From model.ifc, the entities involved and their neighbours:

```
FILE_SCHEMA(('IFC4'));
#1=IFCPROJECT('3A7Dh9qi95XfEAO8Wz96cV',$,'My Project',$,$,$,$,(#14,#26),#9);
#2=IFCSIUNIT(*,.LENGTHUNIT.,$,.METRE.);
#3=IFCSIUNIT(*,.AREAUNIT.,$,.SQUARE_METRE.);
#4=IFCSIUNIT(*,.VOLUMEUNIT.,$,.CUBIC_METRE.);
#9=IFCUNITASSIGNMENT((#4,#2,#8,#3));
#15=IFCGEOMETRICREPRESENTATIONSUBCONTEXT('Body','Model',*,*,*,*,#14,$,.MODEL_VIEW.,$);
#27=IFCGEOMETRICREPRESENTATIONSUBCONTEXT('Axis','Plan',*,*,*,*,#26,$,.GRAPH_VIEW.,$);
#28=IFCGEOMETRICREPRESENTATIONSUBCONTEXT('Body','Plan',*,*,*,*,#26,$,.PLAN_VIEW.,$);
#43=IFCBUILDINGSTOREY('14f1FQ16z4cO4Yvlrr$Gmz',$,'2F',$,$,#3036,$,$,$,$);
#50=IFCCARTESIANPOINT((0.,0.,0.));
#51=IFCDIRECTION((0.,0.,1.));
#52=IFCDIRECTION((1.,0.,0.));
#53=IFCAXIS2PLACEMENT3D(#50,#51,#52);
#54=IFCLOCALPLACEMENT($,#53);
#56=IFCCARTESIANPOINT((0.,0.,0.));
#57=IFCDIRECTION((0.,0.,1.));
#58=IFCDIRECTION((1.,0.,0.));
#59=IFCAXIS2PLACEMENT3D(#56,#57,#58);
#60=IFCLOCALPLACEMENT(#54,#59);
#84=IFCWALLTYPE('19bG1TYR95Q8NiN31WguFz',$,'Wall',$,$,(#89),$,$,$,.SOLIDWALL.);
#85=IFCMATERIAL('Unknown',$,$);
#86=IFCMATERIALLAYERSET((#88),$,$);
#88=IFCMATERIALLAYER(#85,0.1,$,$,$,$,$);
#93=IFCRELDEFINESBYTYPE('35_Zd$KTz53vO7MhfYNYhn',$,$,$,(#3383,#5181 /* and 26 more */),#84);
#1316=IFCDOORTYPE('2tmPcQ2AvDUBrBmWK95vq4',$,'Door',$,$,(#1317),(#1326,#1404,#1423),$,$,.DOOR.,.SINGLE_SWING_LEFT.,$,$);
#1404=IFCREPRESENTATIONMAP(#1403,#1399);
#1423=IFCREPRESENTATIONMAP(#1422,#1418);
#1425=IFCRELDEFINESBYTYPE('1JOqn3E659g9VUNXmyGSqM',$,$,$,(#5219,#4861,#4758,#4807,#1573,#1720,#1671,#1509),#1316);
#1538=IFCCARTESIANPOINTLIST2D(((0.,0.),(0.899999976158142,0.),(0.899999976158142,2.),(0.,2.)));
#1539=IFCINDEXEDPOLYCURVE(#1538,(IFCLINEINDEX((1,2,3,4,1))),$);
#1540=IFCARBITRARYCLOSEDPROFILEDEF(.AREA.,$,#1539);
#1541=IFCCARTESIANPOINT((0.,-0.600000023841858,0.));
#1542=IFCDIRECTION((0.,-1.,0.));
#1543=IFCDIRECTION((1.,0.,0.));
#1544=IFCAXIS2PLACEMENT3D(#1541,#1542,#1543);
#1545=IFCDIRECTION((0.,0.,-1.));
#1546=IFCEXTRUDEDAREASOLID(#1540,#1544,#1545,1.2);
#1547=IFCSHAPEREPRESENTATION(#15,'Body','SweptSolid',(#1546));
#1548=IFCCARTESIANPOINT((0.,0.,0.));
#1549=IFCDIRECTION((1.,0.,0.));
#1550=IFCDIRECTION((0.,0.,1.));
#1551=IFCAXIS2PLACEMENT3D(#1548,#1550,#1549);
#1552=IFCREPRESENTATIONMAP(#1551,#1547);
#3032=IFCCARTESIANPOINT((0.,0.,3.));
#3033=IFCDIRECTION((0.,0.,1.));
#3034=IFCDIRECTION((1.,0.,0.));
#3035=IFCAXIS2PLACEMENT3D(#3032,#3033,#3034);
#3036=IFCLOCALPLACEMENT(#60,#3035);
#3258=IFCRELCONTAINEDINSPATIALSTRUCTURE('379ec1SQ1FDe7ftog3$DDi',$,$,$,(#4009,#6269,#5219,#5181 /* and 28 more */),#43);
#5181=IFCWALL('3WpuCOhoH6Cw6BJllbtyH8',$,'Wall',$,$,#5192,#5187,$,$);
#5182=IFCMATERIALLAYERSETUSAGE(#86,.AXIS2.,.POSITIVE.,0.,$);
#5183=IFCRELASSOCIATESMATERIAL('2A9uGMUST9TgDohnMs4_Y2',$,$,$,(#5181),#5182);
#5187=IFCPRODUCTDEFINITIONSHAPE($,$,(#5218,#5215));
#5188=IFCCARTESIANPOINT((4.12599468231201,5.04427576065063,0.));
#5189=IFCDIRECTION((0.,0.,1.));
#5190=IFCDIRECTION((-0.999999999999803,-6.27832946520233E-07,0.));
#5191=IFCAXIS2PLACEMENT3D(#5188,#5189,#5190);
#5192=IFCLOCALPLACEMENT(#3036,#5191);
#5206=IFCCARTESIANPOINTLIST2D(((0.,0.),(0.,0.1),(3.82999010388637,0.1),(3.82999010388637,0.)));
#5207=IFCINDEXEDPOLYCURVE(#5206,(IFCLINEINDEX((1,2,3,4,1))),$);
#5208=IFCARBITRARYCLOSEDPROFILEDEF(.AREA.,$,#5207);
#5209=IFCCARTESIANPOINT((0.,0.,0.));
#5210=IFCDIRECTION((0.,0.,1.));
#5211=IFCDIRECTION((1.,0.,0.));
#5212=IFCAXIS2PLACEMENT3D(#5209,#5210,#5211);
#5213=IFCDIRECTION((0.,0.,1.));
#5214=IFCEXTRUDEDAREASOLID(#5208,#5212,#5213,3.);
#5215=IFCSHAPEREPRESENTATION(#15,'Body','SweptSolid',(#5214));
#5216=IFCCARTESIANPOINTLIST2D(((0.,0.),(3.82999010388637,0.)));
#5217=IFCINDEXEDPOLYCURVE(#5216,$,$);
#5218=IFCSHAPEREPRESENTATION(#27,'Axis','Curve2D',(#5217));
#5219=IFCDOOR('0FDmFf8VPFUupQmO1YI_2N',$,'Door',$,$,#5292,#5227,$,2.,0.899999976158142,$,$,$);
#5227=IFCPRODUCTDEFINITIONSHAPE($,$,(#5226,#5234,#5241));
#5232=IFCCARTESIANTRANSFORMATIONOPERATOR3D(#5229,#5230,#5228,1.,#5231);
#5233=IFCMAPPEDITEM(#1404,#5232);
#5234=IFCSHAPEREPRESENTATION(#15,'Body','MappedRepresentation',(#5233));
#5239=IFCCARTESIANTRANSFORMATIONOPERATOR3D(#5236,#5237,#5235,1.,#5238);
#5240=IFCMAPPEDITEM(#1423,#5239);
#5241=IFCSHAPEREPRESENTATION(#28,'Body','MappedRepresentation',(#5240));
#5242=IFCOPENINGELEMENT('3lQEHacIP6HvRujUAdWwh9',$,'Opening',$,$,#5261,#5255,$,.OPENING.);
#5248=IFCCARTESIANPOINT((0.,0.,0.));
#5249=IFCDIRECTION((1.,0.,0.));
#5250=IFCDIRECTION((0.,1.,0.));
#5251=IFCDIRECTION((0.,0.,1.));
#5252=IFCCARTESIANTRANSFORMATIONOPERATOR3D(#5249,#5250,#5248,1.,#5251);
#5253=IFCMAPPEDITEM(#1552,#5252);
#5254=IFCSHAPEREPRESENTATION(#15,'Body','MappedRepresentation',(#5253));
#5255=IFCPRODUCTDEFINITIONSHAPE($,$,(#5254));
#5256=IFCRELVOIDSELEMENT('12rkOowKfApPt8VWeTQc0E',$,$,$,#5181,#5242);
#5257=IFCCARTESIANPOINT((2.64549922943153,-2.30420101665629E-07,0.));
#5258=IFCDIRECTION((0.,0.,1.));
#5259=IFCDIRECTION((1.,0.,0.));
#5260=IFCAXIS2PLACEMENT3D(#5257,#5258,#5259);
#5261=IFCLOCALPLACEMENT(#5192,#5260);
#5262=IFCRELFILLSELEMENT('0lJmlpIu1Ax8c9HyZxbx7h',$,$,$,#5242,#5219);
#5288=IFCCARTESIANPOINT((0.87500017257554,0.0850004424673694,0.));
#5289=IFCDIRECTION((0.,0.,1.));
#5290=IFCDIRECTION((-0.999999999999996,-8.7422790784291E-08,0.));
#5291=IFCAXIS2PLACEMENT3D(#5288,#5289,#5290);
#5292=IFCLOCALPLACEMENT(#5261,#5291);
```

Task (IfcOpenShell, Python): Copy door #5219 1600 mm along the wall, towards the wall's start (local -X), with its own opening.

```python
import ifcopenshell
import ifcopenshell.api.feature
import ifcopenshell.api.geometry
import ifcopenshell.api.root
import ifcopenshell.geom
import ifcopenshell.util.element
import ifcopenshell.util.placement
import ifcopenshell.util.shape

model = ifcopenshell.open("model.ifc")
settings = ifcopenshell.geom.settings()


def volume(element):
    """Net volume in cubic metres, openings subtracted."""
    shape = ifcopenshell.geom.create_shape(settings, element)
    return ifcopenshell.util.shape.get_volume(shape.geometry)


door = model.by_guid("0FDmFf8VPFUupQmO1YI_2N")
opening = door.FillsVoids[0].RelatingOpeningElement
wall = opening.VoidsElements[0].RelatingBuildingElement
before = volume(wall)
shift = ifcopenshell.util.placement.get_local_placement(wall.ObjectPlacement)[:3, 0] * -1.6

# copy_class copies the void relationship, type, container and properties, but no geometry.
new_opening = ifcopenshell.api.root.copy_class(model, product=opening)
new_opening.Representation = ifcopenshell.util.element.copy_deep(
    model, opening.Representation, exclude=["IfcGeometricRepresentationContext", "IfcRepresentationMap"]
)
new_door = ifcopenshell.api.root.copy_class(model, product=door)
new_door.Representation = ifcopenshell.util.element.copy_deep(
    model, door.Representation, exclude=["IfcGeometricRepresentationContext", "IfcRepresentationMap"]
)
ifcopenshell.api.feature.add_filling(model, opening=new_opening, element=new_door)

for old, new in ((opening, new_opening), (door, new_door)):
    matrix = ifcopenshell.util.placement.get_local_placement(old.ObjectPlacement)
    matrix[:3, 3] += shift
    ifcopenshell.api.geometry.edit_object_placement(model, product=new, matrix=matrix, is_si=False)

after = volume(wall)

print(f"wall volume {before:.3f} -> {after:.3f} m3")

model.write("model_updated.ifc")
```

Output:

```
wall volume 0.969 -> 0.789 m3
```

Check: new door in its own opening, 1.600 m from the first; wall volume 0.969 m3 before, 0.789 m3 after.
